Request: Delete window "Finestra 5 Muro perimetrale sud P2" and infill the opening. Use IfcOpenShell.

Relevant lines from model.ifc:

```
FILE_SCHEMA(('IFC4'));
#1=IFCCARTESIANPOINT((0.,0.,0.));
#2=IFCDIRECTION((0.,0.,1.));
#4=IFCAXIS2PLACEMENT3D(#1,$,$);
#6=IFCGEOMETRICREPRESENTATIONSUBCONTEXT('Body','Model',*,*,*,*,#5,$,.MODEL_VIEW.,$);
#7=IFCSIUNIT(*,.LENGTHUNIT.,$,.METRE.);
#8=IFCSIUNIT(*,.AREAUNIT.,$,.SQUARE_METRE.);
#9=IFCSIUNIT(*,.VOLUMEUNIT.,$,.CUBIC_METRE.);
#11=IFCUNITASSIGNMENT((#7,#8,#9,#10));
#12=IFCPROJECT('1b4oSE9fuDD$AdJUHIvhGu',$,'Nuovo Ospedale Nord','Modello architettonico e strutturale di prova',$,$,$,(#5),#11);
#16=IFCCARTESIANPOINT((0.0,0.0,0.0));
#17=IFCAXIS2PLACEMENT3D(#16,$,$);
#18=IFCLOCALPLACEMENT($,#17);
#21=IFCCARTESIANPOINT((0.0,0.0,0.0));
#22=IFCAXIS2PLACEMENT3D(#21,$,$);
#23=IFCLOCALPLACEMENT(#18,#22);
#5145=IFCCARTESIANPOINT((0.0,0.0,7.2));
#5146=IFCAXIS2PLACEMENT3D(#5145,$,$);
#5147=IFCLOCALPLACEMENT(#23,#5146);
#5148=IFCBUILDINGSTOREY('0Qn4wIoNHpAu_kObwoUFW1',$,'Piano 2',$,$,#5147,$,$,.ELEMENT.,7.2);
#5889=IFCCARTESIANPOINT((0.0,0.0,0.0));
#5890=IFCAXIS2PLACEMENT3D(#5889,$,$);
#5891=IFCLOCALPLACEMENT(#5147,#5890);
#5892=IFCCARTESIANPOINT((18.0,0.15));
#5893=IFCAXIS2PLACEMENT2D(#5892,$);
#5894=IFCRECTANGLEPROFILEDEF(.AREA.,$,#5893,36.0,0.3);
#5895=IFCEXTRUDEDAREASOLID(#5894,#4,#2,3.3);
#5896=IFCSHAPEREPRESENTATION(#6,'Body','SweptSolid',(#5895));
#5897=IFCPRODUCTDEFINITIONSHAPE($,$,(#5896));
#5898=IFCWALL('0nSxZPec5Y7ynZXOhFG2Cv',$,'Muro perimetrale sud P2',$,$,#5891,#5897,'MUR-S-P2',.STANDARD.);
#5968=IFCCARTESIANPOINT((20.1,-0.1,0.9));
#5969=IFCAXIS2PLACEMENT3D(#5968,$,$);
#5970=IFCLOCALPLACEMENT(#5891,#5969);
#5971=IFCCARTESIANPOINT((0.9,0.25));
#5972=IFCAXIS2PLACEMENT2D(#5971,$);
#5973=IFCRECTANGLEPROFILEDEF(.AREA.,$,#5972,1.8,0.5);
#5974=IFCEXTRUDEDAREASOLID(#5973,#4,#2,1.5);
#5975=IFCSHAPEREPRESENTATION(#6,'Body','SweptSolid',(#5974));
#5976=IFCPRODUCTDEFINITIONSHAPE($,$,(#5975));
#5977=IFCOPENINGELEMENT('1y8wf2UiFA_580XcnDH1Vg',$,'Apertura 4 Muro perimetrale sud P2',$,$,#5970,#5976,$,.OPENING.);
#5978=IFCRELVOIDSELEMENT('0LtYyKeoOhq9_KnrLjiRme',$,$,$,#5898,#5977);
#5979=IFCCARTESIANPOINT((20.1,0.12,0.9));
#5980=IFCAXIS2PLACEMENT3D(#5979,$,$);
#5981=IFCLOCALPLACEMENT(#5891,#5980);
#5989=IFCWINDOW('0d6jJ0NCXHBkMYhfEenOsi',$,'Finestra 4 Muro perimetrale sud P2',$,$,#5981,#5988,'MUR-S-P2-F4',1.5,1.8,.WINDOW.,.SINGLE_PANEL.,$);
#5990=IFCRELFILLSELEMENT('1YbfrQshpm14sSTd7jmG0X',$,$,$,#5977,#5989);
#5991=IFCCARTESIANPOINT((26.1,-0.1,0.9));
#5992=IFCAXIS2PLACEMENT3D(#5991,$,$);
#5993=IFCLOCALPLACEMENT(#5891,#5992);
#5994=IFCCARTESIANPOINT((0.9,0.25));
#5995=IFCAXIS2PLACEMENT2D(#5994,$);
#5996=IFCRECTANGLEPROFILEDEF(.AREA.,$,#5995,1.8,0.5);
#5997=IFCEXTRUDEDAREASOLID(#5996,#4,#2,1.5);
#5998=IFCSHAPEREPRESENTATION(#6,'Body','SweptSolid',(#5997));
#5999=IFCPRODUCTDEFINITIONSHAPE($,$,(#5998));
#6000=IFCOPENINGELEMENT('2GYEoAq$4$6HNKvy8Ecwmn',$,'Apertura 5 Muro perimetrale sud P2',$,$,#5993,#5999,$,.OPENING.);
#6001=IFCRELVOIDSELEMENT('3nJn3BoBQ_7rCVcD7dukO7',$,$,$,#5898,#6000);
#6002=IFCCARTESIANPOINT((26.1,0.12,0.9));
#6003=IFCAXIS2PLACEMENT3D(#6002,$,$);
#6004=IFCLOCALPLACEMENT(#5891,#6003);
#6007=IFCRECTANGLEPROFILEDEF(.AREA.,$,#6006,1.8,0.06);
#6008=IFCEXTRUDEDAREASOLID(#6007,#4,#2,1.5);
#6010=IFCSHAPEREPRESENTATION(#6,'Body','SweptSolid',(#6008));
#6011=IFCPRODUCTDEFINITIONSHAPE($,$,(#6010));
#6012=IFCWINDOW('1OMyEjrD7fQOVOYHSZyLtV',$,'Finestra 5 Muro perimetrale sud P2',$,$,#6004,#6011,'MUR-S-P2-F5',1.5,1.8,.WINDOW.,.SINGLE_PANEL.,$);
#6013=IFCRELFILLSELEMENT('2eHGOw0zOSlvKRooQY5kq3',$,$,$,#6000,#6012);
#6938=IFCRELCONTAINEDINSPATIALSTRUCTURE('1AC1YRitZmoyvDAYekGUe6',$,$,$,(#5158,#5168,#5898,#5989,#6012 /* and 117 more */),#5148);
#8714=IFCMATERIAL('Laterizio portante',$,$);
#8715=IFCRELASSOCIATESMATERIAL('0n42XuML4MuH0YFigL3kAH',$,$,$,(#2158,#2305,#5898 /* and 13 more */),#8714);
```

```python
import ifcopenshell
import ifcopenshell.api.feature
import ifcopenshell.api.root
import ifcopenshell.geom
import ifcopenshell.util.shape

model = ifcopenshell.open("model.ifc")
settings = ifcopenshell.geom.settings()


def volume(element):
    """Net volume in cubic metres, openings subtracted."""
    shape = ifcopenshell.geom.create_shape(settings, element)
    return ifcopenshell.util.shape.get_volume(shape.geometry)


window = model.by_id(6012)
opening = window.FillsVoids[0].RelatingOpeningElement
wall = opening.VoidsElements[0].RelatingBuildingElement
before = volume(wall)

ifcopenshell.api.root.remove_product(model, product=window)
ifcopenshell.api.feature.remove_feature(model, feature=opening)

after = volume(wall)

print(f"wall volume {before:.3f} -> {after:.3f} m3")

model.write("model_rev.ifc")
```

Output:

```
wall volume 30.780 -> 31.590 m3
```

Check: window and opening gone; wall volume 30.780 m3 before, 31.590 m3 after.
